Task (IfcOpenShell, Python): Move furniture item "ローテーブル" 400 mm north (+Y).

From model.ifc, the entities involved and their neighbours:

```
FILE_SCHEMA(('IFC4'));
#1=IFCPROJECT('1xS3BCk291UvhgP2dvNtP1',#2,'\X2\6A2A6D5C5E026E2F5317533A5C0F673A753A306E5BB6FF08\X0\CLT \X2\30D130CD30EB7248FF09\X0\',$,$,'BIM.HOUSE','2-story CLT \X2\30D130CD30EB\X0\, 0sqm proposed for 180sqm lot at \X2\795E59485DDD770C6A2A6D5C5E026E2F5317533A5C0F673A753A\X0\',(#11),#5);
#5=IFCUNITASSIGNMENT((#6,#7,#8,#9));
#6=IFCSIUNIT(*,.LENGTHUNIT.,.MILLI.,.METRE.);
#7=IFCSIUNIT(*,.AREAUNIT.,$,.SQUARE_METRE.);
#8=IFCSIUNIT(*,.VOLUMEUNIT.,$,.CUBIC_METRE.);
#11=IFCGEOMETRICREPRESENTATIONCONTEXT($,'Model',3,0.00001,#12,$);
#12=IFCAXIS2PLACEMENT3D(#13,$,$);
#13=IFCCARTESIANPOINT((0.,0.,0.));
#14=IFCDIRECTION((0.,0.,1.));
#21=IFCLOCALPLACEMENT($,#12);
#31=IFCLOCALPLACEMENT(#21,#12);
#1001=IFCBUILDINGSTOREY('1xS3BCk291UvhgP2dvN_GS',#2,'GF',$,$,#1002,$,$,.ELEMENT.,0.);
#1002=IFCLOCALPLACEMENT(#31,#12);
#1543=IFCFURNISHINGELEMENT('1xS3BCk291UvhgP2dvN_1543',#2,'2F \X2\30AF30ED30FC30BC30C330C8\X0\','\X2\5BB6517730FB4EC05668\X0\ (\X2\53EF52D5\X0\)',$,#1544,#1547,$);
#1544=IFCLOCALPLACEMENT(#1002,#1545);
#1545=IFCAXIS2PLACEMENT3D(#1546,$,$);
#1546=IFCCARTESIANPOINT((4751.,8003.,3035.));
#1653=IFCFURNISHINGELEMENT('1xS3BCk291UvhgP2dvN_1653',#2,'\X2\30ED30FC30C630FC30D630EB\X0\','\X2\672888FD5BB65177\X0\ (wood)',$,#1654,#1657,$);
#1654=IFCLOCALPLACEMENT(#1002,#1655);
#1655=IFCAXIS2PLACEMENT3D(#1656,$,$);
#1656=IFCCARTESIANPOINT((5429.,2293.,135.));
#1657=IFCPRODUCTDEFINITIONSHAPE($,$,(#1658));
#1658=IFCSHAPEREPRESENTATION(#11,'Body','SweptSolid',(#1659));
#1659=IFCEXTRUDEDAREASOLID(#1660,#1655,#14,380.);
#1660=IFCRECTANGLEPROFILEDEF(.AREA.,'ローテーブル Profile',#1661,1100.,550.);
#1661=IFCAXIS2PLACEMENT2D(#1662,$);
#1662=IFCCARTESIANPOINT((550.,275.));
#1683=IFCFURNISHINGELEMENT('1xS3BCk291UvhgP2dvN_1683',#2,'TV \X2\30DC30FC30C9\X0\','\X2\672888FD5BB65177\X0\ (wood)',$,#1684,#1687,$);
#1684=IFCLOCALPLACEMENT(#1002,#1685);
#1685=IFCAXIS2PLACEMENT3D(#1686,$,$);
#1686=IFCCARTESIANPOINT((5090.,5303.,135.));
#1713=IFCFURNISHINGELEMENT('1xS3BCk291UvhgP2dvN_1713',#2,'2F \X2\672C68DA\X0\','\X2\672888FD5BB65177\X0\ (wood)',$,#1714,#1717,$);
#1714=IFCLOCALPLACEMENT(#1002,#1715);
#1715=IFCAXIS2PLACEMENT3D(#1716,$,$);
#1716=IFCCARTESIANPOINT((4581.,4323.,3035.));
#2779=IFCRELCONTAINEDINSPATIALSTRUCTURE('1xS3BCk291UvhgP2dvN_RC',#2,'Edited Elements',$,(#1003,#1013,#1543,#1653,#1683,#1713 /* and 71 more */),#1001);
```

```python
import ifcopenshell
import ifcopenshell.api.geometry
import ifcopenshell.util.placement
import ifcopenshell.util.unit

model = ifcopenshell.open("model.ifc")
unit_scale = ifcopenshell.util.unit.calculate_unit_scale(model)

item = model.by_id(1653)
matrix = ifcopenshell.util.placement.get_local_placement(item.ObjectPlacement)
matrix[1, 3] += 0.4 / unit_scale
ifcopenshell.api.geometry.edit_object_placement(model, product=item, matrix=matrix, is_si=False)

print(ifcopenshell.util.placement.get_local_placement(item.ObjectPlacement).round(3) + 0.0)

model.write("model_updated.ifc")
```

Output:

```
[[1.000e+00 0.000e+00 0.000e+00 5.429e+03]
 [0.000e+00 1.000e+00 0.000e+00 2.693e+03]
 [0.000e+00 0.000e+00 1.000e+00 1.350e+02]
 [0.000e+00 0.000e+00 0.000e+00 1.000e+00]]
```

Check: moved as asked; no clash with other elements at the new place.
